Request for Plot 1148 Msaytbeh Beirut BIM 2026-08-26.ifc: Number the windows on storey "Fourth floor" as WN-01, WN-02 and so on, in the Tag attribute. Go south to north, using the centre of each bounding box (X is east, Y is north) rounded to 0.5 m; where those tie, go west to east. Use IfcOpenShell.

First a look at what the model holds.

```python
import ifcopenshell
import ifcopenshell.util.element
import ifcopenshell.util.placement

model = ifcopenshell.open("Plot 1148 Msaytbeh Beirut BIM 2026-08-26.ifc")
print(model.schema)
storey = next(s for s in model.by_type("IfcBuildingStorey") if s.Name == "Fourth floor")
windows = [e for e in ifcopenshell.util.element.get_decomposition(storey) if e.is_a("IfcWindow")]
for e in sorted(windows, key=lambda e: e.id()):
    origin = ifcopenshell.util.placement.get_local_placement(e.ObjectPlacement)[:3, 3]
    print(e.id(), e.Tag, e.Name, origin.round(2) + 0.0, sep=" | ")
```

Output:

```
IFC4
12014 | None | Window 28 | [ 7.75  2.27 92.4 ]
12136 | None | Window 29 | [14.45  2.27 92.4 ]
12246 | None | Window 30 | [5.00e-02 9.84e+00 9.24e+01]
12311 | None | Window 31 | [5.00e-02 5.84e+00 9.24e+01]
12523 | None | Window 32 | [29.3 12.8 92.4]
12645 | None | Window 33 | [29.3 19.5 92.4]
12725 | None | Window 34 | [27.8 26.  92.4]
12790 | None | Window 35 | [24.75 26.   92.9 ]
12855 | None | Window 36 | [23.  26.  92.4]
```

```python
import ifcopenshell
import ifcopenshell.geom
import ifcopenshell.util.element
import ifcopenshell.util.shape

model = ifcopenshell.open("Plot 1148 Msaytbeh Beirut BIM 2026-08-26.ifc")
settings = ifcopenshell.geom.settings()
settings.set("use-world-coords", True)


def centre(element):
    shape = ifcopenshell.geom.create_shape(settings, element)
    return ifcopenshell.util.shape.get_bbox_centroid(shape.geometry)


storey = next(s for s in model.by_type("IfcBuildingStorey") if s.Name == "Fourth floor")
windows = [e for e in ifcopenshell.util.element.get_decomposition(storey) if e.is_a("IfcWindow")]

# Insertion points can sit at a corner or the storey origin, so sort by the geometry (in metres).
centres = {e: centre(e) for e in windows}
windows.sort(key=lambda e: (round(centres[e][1] / 0.5), centres[e][0]))

for i, e in enumerate(windows, start=1):
    number = f"WN-{i:02d}"
    e.Tag = number
    print(e.id(), number)

model.write("Plot 1148 Msaytbeh Beirut BIM 2026-08-26_rev.ifc")
```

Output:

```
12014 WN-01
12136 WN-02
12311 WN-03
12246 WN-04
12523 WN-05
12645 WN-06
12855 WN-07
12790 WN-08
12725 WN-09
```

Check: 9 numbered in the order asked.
